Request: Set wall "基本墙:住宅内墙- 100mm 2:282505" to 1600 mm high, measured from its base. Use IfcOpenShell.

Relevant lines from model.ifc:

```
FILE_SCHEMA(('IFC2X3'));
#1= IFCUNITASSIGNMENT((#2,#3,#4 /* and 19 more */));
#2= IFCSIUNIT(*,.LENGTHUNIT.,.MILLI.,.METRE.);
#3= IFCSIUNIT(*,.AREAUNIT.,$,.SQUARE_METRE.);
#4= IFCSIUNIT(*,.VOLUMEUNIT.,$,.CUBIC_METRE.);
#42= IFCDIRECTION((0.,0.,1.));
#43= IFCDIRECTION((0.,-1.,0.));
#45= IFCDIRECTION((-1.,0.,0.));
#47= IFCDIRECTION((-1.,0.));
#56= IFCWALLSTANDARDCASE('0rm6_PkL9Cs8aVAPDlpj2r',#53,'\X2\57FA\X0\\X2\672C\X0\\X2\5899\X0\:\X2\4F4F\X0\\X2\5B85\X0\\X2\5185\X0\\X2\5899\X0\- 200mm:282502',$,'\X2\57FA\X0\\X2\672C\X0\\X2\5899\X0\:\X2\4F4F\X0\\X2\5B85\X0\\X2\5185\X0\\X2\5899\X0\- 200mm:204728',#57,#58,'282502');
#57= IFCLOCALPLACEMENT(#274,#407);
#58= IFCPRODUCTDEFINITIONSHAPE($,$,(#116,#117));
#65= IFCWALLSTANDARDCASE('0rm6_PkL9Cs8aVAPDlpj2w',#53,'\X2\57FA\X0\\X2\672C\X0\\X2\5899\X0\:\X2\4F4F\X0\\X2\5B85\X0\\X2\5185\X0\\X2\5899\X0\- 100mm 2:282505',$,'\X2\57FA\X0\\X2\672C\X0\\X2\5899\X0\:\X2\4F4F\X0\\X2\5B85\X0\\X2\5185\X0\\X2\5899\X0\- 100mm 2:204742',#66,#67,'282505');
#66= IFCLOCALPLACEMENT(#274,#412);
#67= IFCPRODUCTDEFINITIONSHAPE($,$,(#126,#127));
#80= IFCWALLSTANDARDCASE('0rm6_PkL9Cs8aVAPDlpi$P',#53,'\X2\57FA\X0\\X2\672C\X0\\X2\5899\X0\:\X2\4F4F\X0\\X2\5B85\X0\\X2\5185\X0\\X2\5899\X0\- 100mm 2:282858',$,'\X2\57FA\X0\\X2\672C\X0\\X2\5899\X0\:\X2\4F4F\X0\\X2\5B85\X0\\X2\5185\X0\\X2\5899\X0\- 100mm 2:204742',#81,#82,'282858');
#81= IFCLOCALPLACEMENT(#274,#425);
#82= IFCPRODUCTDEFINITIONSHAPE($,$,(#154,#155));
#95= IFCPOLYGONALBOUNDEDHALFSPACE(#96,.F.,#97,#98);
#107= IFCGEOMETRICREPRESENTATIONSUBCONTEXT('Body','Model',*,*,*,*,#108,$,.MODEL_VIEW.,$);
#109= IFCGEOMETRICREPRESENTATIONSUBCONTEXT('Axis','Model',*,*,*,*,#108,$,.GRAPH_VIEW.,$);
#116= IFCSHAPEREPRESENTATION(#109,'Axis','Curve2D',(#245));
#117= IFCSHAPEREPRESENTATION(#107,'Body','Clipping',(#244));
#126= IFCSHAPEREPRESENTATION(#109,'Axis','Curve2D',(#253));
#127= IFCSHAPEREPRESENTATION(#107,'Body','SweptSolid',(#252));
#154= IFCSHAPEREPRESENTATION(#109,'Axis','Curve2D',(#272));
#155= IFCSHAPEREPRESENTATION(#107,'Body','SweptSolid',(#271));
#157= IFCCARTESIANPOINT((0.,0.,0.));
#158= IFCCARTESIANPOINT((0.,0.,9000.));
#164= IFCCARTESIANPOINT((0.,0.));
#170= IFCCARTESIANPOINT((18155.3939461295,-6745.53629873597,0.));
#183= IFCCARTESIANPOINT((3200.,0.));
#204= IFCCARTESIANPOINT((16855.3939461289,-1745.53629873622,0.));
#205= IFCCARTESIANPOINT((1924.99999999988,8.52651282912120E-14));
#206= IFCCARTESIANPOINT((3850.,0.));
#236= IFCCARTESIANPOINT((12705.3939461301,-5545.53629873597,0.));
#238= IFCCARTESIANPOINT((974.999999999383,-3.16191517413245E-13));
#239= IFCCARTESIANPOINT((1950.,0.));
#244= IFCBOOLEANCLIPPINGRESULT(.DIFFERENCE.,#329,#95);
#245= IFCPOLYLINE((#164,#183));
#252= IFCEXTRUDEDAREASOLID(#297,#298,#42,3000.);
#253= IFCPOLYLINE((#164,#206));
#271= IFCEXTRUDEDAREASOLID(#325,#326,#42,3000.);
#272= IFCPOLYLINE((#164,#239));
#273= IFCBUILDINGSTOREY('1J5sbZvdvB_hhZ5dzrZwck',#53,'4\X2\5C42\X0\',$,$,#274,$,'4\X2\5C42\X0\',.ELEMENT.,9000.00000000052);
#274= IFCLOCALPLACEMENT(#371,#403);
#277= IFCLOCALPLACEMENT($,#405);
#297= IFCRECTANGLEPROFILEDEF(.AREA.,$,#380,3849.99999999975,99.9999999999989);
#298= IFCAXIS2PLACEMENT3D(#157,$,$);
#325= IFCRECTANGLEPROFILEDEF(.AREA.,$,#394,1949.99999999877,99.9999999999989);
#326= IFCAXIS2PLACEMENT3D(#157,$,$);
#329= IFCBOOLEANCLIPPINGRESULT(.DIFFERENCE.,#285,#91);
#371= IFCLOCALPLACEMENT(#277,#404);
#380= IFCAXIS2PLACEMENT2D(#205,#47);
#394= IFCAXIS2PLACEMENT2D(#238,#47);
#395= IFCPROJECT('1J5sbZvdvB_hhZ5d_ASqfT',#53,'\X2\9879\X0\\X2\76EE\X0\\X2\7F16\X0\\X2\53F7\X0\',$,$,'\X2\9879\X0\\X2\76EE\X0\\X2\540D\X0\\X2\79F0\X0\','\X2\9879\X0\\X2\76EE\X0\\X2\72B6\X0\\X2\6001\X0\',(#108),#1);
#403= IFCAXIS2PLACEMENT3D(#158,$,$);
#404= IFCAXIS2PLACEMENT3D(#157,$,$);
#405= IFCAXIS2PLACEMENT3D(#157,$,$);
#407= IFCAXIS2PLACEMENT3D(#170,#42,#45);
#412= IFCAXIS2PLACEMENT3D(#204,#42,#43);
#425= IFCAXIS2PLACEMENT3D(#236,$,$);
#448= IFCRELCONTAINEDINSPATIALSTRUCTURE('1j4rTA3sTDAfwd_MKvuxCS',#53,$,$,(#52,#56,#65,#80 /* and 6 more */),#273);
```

```python
import ifcopenshell
import ifcopenshell.geom
import ifcopenshell.util.representation
import ifcopenshell.util.shape

model = ifcopenshell.open("model.ifc")
settings = ifcopenshell.geom.settings()


def volume(element):
    """Net volume in cubic metres, openings subtracted."""
    shape = ifcopenshell.geom.create_shape(settings, element)
    return ifcopenshell.util.shape.get_volume(shape.geometry)


wall = model.by_guid("0rm6_PkL9Cs8aVAPDlpj2w")
before = volume(wall)

body = ifcopenshell.util.representation.get_representation(wall, "Model", "Body")
solid = body.Items[0]
old_height = solid.Depth
solid.Depth = 1600.0
after = volume(wall)

print(f"height {old_height:g} -> {solid.Depth:g}, volume {before:.3f} -> {after:.3f} m3")

model.write("model-out.ifc")
```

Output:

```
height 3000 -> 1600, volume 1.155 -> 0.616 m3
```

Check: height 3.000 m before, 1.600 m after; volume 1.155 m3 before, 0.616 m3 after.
